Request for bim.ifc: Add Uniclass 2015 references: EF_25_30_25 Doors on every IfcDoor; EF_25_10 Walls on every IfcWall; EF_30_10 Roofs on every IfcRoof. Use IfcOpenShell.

First a look at what the model holds.

```python
import ifcopenshell

model = ifcopenshell.open("bim.ifc")
print(model.schema)
print("classifications:", [c.Name for c in model.by_type("IfcClassification")])
for ifc_class in ("IfcDoor", "IfcRoof", "IfcStair", "IfcWall", "IfcWindow"):
    print(ifc_class, len(model.by_type(ifc_class)))
```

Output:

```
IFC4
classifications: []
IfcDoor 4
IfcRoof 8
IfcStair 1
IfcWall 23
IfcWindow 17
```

```python
import ifcopenshell
import ifcopenshell.api.classification

model = ifcopenshell.open("bim.ifc")

system = ifcopenshell.api.classification.add_classification(model, classification="Uniclass 2015")

codes = {
    "IfcDoor": ("EF_25_30_25", "Doors"),
    "IfcWall": ("EF_25_10", "Walls"),
    "IfcRoof": ("EF_30_10", "Roofs"),
}
for ifc_class, (code, name) in codes.items():
    products = model.by_type(ifc_class)
    ifcopenshell.api.classification.add_reference(
        model, products=products, classification=system, identification=code, name=name
    )
    print(code, len(products))

model.write("bim_edited.ifc")
```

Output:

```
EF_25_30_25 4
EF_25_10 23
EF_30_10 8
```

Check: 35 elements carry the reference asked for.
